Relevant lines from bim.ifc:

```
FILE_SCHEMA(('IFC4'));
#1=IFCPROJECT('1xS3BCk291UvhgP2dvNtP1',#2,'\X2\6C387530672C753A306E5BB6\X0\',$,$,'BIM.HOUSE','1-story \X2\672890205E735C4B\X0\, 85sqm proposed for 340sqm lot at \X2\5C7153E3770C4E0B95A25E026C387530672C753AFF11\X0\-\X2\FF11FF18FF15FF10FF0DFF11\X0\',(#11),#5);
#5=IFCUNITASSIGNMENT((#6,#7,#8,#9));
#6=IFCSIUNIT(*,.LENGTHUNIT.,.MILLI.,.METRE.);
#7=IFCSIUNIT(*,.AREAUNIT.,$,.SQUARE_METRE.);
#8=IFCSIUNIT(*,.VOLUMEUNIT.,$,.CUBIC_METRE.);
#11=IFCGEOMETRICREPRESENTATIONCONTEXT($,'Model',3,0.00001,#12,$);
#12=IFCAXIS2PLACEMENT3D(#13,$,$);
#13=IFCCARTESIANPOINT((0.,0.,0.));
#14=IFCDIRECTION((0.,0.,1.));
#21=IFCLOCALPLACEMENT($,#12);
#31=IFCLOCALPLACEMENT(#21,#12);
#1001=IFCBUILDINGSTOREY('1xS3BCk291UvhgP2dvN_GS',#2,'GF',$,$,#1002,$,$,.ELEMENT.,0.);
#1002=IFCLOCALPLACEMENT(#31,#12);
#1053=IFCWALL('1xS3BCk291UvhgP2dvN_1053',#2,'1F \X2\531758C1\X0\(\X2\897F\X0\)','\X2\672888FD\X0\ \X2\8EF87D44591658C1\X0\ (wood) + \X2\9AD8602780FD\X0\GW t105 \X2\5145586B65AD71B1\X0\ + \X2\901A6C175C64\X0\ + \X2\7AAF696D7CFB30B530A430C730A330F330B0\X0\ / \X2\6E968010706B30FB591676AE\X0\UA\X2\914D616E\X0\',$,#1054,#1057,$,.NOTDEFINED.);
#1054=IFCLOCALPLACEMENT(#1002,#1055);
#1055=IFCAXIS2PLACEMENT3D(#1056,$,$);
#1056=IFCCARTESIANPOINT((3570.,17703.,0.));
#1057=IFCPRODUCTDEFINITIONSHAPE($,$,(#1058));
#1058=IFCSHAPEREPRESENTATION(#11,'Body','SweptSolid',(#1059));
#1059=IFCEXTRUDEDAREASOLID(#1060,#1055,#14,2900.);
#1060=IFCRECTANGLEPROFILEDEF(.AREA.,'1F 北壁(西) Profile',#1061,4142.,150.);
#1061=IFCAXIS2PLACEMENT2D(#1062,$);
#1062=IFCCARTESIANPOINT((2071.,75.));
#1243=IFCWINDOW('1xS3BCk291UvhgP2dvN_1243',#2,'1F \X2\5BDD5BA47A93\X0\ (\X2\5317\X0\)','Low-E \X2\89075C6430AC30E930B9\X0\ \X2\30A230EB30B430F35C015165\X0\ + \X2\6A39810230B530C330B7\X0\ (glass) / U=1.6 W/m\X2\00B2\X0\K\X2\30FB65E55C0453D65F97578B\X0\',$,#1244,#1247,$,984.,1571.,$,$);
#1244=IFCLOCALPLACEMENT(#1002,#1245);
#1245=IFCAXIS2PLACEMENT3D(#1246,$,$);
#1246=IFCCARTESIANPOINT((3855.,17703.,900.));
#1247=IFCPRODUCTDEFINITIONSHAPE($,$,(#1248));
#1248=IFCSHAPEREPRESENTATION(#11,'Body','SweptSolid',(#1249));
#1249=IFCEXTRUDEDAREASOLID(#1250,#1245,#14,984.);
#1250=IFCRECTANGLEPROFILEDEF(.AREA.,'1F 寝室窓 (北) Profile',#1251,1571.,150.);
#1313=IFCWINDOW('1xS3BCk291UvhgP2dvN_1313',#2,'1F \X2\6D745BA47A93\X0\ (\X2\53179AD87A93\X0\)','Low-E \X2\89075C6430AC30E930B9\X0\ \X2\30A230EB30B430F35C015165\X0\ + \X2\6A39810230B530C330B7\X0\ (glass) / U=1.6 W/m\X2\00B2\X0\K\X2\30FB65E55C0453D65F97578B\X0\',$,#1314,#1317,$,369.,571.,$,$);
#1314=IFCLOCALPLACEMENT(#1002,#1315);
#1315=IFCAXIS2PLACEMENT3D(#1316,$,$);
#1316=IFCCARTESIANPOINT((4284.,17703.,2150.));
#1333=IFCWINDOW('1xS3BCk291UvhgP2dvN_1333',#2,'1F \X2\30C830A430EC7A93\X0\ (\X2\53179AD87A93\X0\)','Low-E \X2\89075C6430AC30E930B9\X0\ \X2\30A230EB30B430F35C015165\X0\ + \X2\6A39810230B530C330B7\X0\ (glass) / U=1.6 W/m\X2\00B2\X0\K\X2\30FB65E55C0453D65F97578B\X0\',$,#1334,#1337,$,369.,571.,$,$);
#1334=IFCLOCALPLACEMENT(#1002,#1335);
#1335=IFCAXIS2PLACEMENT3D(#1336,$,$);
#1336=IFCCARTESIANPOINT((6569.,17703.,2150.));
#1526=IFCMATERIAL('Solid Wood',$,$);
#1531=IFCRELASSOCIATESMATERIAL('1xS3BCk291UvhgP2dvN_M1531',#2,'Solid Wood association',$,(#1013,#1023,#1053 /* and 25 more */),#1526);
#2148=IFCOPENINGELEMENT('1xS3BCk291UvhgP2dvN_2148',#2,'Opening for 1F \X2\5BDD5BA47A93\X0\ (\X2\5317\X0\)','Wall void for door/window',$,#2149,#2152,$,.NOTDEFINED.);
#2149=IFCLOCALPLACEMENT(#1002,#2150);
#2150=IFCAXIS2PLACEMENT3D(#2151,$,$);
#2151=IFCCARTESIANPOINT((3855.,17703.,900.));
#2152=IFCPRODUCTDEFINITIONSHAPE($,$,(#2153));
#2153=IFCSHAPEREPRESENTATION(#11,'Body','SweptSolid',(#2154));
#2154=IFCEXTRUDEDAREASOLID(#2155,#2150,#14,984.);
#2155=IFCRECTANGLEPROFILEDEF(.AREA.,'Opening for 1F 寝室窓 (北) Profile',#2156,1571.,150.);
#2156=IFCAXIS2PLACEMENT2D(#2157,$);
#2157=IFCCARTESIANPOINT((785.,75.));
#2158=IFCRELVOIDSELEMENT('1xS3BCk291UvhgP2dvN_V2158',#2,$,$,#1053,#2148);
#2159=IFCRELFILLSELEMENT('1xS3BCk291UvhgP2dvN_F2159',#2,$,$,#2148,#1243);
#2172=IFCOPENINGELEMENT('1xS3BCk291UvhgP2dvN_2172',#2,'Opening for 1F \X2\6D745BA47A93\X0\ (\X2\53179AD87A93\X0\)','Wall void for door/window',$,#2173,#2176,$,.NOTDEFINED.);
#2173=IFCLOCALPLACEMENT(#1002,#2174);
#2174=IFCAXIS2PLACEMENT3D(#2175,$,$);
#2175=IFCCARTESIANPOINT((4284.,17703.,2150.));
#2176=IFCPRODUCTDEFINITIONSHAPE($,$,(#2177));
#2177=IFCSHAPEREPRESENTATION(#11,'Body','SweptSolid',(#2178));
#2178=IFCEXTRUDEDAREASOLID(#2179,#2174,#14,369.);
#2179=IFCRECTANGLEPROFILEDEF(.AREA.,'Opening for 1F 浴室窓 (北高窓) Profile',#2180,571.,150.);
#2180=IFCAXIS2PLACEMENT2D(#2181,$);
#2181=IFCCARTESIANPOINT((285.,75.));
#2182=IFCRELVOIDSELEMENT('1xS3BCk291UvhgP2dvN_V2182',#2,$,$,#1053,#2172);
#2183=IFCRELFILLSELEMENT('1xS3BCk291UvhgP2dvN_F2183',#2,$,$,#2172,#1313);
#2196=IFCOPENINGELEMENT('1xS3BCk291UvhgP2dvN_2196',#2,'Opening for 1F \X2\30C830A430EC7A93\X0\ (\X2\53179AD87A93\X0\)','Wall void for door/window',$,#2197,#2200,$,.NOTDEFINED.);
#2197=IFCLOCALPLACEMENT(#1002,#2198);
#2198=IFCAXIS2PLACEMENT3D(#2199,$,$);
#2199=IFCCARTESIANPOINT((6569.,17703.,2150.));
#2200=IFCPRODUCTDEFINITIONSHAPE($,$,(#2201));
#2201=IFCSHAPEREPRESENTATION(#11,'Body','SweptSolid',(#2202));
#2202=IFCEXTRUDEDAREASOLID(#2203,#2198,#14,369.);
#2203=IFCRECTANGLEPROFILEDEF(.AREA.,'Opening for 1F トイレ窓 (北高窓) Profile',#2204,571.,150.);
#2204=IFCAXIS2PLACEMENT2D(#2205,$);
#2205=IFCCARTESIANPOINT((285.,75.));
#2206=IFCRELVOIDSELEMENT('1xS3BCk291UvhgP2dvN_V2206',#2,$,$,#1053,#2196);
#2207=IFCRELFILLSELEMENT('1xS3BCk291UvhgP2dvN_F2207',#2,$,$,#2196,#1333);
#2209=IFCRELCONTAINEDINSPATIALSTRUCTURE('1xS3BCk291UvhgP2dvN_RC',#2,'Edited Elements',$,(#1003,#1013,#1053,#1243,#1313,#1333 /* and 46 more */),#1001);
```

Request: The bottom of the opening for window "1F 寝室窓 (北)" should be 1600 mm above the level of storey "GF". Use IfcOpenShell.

```python
import numpy as np
import ifcopenshell
import ifcopenshell.api.geometry
import ifcopenshell.geom
import ifcopenshell.util.element
import ifcopenshell.util.placement
import ifcopenshell.util.shape
import ifcopenshell.util.unit

model = ifcopenshell.open("bim.ifc")
unit_scale = ifcopenshell.util.unit.calculate_unit_scale(model)

window = model.by_guid("1xS3BCk291UvhgP2dvN_1243")
opening = window.FillsVoids[0].RelatingOpeningElement
storey = ifcopenshell.util.element.get_container(window, ifc_class="IfcBuildingStorey")
level = ifcopenshell.util.placement.get_local_placement(storey.ObjectPlacement)[2, 3]

# The opening's origin need not be at the sill, so measure its lowest point.
shape = ifcopenshell.geom.create_shape(ifcopenshell.geom.settings(), opening)
bottom = ifcopenshell.util.shape.get_shape_bottom_elevation(shape, shape.geometry) / unit_scale
dz = level + 1.6 / unit_scale - bottom

shift = np.array([0.0, 0.0, dz])
# The window is not placed relative to its opening, so move both.
for product in (opening, window):
    matrix = ifcopenshell.util.placement.get_local_placement(product.ObjectPlacement)
    matrix[:3, 3] += shift
    ifcopenshell.api.geometry.edit_object_placement(model, product=product, matrix=matrix, is_si=False)

print(f"moved by {dz * unit_scale:+.3f} m")

model.write("bim-out.ifc")
```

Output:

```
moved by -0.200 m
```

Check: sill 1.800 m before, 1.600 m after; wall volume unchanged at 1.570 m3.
